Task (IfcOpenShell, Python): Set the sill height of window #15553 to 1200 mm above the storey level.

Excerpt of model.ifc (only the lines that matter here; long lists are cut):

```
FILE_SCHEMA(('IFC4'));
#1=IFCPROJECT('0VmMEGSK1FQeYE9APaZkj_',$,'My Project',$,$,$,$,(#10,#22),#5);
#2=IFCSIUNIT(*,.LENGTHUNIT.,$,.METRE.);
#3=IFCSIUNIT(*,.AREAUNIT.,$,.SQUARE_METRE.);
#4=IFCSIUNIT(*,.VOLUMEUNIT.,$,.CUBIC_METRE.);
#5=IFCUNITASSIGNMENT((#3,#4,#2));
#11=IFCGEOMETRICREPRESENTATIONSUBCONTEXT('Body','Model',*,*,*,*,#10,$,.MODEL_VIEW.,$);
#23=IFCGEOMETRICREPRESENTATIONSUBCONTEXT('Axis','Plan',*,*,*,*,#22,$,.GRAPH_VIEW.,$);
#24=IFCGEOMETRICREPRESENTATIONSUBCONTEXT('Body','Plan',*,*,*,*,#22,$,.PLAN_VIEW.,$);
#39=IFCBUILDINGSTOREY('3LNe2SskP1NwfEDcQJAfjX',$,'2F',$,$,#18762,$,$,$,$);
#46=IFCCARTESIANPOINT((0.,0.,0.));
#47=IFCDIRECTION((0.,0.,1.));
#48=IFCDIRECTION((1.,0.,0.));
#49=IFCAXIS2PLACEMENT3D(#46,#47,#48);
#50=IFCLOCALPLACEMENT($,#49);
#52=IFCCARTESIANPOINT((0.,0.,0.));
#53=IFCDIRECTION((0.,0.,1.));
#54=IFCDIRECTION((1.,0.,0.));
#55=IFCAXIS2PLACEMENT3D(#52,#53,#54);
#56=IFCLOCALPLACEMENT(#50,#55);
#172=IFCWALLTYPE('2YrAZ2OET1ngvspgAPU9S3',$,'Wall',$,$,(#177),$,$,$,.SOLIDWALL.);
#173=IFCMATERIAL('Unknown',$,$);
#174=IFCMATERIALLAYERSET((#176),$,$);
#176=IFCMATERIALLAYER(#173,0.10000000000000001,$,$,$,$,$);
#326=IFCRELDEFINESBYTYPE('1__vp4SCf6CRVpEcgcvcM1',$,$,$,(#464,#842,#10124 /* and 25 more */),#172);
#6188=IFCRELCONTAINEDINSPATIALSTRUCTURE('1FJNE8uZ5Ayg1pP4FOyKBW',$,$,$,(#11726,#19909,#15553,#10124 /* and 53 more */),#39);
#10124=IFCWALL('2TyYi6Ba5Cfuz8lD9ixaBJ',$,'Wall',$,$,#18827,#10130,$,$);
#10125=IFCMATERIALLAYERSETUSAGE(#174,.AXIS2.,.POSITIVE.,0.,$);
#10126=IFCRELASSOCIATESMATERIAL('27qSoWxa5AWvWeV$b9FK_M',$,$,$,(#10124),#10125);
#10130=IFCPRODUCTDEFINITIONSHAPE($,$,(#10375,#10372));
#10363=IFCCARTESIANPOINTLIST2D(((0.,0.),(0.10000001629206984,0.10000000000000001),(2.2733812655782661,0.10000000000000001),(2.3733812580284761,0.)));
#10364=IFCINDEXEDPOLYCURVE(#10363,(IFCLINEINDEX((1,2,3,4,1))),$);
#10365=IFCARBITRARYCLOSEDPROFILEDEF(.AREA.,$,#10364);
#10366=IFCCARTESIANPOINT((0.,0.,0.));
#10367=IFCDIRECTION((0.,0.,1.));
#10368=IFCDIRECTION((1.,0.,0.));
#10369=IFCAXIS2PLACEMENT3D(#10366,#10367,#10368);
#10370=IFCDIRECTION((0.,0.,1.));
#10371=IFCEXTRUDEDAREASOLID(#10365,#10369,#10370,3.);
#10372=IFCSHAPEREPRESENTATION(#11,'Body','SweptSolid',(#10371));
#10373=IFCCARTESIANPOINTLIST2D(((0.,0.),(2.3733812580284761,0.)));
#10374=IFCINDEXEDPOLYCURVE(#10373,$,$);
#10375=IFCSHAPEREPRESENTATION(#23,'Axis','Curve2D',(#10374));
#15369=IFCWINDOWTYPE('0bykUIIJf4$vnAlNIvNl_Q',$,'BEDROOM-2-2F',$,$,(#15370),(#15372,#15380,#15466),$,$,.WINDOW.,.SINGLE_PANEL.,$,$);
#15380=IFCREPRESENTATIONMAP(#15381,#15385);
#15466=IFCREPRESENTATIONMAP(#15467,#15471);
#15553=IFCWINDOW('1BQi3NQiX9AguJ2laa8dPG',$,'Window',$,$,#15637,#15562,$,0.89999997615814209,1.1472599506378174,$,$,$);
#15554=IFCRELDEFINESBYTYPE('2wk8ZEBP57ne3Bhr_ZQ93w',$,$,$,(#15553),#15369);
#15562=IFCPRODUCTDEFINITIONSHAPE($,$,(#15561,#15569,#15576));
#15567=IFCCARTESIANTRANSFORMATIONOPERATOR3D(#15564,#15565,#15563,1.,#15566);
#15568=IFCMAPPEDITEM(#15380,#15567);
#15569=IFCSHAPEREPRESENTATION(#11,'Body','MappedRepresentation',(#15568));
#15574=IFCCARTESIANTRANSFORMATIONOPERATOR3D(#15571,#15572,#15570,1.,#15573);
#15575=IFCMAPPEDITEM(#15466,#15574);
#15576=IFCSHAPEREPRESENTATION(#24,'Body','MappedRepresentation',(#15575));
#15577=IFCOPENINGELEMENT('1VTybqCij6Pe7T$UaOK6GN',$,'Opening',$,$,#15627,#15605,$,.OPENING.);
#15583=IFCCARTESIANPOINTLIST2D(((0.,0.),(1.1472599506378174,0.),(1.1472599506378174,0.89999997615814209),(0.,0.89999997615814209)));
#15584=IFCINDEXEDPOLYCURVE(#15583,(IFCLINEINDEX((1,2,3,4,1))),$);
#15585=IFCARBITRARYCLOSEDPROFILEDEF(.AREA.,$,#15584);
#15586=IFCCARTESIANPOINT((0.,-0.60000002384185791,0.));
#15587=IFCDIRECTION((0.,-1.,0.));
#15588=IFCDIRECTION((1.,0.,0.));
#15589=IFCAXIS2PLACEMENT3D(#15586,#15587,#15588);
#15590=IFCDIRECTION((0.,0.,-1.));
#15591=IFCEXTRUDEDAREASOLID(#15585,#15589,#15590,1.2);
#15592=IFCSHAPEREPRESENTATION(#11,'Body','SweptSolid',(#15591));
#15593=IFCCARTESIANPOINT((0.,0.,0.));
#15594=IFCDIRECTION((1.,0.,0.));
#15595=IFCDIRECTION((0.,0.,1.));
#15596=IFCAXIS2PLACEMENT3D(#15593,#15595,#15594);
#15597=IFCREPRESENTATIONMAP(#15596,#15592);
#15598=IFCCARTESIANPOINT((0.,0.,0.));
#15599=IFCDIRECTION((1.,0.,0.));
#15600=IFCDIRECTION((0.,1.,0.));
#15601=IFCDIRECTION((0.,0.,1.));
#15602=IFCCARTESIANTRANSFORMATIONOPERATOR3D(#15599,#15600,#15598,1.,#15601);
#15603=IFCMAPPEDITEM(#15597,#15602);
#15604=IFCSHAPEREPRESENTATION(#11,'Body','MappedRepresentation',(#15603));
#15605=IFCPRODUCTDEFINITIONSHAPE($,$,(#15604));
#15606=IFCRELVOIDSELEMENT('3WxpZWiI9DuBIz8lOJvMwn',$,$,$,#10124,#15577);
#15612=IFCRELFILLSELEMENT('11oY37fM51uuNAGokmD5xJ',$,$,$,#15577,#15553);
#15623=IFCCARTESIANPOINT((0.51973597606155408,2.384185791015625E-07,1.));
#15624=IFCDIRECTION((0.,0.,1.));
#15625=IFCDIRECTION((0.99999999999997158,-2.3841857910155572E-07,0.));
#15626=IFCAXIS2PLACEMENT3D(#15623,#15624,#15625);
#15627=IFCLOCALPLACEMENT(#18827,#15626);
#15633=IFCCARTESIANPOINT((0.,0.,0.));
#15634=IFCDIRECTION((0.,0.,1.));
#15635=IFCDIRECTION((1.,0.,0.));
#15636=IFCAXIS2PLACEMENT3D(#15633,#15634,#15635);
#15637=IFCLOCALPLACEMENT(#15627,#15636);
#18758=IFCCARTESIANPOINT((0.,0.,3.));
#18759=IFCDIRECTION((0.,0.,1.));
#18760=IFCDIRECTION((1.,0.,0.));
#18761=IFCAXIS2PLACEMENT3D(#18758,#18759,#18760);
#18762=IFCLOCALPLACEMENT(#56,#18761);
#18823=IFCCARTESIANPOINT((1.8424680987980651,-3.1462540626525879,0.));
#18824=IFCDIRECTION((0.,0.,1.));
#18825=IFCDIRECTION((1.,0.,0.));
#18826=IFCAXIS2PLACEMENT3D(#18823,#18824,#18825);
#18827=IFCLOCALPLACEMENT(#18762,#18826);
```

```python
import numpy as np
import ifcopenshell
import ifcopenshell.api.geometry
import ifcopenshell.geom
import ifcopenshell.util.element
import ifcopenshell.util.placement
import ifcopenshell.util.shape
import ifcopenshell.util.unit

model = ifcopenshell.open("model.ifc")
unit_scale = ifcopenshell.util.unit.calculate_unit_scale(model)

window = model.by_guid("1BQi3NQiX9AguJ2laa8dPG")
opening = window.FillsVoids[0].RelatingOpeningElement
storey = ifcopenshell.util.element.get_container(window, ifc_class="IfcBuildingStorey")
level = ifcopenshell.util.placement.get_local_placement(storey.ObjectPlacement)[2, 3]

# The opening's origin need not be at the sill, so measure its lowest point.
shape = ifcopenshell.geom.create_shape(ifcopenshell.geom.settings(), opening)
bottom = ifcopenshell.util.shape.get_shape_bottom_elevation(shape, shape.geometry) / unit_scale
dz = level + 1.2 - bottom

shift = np.array([0.0, 0.0, dz])
# The window is placed relative to its opening, so it follows when the opening moves.
matrix = ifcopenshell.util.placement.get_local_placement(opening.ObjectPlacement)
matrix[:3, 3] += shift
ifcopenshell.api.geometry.edit_object_placement(
    model, product=opening, matrix=matrix, is_si=False, should_transform_children=True
)

print(f"moved by {dz * unit_scale:+.3f} m")

model.write("model_updated.ifc")
```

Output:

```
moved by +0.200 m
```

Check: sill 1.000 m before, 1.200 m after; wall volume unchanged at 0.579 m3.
